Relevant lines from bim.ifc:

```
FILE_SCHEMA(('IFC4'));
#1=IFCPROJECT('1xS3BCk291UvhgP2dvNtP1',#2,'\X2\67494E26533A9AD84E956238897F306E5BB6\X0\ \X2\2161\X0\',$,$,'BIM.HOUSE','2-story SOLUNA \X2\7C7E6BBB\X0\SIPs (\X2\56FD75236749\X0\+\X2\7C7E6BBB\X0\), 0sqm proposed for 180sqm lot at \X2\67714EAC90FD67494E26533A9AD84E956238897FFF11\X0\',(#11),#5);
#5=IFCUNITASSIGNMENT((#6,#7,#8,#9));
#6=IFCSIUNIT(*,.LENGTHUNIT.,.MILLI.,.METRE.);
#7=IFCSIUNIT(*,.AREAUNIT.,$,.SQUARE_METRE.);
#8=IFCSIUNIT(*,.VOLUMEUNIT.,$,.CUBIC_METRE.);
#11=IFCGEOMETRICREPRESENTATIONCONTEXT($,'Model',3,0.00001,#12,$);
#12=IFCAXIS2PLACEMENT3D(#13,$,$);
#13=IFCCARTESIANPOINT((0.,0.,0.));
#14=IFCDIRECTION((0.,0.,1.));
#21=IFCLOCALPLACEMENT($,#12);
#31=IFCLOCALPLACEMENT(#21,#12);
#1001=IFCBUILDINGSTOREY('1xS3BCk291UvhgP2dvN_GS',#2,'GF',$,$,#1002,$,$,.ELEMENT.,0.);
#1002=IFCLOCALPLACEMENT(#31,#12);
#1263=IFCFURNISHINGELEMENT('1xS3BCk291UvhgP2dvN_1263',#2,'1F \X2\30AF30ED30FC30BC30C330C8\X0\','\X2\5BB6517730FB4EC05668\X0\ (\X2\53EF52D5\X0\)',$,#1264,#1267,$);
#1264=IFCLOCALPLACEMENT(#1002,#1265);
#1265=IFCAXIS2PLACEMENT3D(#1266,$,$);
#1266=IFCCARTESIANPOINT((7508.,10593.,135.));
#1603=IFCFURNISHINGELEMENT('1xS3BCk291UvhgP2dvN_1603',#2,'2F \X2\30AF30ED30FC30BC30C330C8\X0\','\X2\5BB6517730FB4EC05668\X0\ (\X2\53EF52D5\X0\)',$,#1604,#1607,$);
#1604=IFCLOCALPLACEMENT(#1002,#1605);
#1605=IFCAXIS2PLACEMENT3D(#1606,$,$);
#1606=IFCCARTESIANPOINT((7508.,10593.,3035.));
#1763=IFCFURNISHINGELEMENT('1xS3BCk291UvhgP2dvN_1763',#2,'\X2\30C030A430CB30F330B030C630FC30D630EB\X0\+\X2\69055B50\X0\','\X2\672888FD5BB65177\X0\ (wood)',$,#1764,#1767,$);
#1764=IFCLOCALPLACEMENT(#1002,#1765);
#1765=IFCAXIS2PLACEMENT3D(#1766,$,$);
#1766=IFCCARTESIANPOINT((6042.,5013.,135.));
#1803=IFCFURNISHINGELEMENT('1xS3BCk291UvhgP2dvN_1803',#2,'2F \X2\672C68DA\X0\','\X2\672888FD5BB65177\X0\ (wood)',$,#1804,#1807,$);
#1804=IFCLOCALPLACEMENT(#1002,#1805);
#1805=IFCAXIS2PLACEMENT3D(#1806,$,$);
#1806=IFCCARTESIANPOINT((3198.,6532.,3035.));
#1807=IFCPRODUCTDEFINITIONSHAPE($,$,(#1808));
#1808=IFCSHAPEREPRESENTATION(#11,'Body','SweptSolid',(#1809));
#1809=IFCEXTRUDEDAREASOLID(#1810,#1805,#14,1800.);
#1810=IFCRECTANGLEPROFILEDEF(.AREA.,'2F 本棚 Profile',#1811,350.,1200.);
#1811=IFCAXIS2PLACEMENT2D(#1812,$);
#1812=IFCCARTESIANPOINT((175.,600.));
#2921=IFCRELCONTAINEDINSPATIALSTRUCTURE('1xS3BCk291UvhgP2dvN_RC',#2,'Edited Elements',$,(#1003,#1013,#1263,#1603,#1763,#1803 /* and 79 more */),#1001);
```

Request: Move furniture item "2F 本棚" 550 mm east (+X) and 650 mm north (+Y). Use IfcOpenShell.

```python
import ifcopenshell
import ifcopenshell.api.geometry
import ifcopenshell.util.placement

model = ifcopenshell.open("bim.ifc")

item = model.by_guid("1xS3BCk291UvhgP2dvN_1803")
matrix = ifcopenshell.util.placement.get_local_placement(item.ObjectPlacement)
matrix[0, 3] += 550.0
matrix[1, 3] += 650.0
ifcopenshell.api.geometry.edit_object_placement(model, product=item, matrix=matrix, is_si=False)

print(ifcopenshell.util.placement.get_local_placement(item.ObjectPlacement).round(3) + 0.0)

model.write("bim_updated.ifc")
```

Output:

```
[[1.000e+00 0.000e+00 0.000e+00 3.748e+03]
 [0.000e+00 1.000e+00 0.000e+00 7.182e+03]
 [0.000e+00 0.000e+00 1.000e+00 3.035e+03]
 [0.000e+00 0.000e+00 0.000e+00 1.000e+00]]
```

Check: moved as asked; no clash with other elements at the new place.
